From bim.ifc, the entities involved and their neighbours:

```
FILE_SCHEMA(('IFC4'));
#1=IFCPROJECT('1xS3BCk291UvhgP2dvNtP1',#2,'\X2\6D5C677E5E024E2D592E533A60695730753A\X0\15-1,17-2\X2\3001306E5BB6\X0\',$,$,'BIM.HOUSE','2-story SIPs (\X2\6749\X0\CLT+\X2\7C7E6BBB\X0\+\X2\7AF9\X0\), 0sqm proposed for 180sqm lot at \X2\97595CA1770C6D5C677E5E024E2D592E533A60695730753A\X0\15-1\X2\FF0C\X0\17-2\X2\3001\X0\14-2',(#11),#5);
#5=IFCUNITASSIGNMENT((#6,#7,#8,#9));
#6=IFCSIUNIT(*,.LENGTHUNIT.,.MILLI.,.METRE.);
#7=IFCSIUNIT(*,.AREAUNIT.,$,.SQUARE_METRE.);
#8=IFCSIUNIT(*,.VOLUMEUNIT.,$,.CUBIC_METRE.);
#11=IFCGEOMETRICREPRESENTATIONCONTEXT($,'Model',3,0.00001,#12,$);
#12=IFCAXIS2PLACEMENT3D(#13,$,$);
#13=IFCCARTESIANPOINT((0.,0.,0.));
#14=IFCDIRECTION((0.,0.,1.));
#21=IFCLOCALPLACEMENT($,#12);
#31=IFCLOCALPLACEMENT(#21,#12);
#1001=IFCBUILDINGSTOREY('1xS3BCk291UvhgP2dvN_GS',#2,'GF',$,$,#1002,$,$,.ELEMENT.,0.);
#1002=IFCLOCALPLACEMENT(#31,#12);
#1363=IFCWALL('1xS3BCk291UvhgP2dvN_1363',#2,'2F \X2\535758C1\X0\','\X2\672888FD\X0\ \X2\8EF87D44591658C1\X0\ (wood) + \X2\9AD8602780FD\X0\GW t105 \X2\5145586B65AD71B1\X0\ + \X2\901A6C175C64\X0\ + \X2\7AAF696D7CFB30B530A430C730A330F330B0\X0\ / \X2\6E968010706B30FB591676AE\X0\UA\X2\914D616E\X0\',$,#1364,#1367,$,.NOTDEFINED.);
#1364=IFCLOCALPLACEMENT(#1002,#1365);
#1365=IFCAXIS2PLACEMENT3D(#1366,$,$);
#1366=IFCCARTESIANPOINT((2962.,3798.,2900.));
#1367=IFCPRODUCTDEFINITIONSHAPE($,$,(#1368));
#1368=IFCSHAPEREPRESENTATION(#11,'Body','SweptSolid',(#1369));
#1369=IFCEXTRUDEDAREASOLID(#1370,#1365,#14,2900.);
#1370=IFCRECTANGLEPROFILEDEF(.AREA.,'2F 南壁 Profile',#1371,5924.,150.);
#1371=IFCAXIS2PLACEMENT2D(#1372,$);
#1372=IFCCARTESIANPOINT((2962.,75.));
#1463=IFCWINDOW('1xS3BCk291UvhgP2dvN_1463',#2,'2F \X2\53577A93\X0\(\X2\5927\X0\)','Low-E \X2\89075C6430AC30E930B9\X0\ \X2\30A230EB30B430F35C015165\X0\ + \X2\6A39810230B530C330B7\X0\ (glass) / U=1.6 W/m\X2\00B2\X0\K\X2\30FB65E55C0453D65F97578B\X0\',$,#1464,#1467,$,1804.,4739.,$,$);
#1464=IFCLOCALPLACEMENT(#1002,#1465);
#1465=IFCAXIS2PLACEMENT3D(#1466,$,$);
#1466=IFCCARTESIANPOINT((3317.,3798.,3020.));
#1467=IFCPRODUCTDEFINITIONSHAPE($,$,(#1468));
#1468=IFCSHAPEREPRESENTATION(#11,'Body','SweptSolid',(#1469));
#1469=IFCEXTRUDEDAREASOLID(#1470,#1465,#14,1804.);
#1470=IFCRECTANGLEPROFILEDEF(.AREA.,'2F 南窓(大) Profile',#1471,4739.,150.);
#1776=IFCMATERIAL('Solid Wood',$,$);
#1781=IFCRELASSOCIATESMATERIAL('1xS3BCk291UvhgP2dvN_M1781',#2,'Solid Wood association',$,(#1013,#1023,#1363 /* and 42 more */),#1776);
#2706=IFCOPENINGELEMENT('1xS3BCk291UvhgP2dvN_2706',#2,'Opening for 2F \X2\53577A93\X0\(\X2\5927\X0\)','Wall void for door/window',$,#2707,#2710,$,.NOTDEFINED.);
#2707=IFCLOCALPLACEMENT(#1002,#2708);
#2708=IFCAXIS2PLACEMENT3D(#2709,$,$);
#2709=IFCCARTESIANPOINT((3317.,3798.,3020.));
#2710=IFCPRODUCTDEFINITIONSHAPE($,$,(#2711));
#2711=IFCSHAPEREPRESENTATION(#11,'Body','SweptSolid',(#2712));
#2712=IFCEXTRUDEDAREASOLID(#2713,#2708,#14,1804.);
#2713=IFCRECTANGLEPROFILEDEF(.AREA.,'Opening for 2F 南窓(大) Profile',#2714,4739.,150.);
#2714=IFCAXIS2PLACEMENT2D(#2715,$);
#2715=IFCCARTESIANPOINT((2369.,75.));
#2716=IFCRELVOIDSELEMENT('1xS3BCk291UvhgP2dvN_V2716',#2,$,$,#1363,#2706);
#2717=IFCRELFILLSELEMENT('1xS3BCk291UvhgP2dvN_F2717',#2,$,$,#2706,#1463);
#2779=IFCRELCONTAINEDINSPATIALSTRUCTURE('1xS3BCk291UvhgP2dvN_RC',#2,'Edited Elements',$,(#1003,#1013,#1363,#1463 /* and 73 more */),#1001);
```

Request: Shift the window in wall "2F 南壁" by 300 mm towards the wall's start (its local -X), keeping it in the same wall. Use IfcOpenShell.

```python
import ifcopenshell
import ifcopenshell.api.geometry
import ifcopenshell.util.placement
import ifcopenshell.util.unit

model = ifcopenshell.open("bim.ifc")
unit_scale = ifcopenshell.util.unit.calculate_unit_scale(model)

window = model.by_guid("1xS3BCk291UvhgP2dvN_1463")
opening = window.FillsVoids[0].RelatingOpeningElement
wall = opening.VoidsElements[0].RelatingBuildingElement

wall_matrix = ifcopenshell.util.placement.get_local_placement(wall.ObjectPlacement)
shift = wall_matrix[:3, 0] * -0.3 / unit_scale
before = ifcopenshell.util.placement.get_local_placement(window.ObjectPlacement)[:3, 3].copy()

# The window is not placed relative to its opening, so move both.
for product in (opening, window):
    matrix = ifcopenshell.util.placement.get_local_placement(product.ObjectPlacement)
    matrix[:3, 3] += shift
    ifcopenshell.api.geometry.edit_object_placement(model, product=product, matrix=matrix, is_si=False)

after = ifcopenshell.util.placement.get_local_placement(window.ObjectPlacement)[:3, 3]
print("window moved by", (after - before).round(3) + 0.0)

model.write("bim_edited.ifc")
```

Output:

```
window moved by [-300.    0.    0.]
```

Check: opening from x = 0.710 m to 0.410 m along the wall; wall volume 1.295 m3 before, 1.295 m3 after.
